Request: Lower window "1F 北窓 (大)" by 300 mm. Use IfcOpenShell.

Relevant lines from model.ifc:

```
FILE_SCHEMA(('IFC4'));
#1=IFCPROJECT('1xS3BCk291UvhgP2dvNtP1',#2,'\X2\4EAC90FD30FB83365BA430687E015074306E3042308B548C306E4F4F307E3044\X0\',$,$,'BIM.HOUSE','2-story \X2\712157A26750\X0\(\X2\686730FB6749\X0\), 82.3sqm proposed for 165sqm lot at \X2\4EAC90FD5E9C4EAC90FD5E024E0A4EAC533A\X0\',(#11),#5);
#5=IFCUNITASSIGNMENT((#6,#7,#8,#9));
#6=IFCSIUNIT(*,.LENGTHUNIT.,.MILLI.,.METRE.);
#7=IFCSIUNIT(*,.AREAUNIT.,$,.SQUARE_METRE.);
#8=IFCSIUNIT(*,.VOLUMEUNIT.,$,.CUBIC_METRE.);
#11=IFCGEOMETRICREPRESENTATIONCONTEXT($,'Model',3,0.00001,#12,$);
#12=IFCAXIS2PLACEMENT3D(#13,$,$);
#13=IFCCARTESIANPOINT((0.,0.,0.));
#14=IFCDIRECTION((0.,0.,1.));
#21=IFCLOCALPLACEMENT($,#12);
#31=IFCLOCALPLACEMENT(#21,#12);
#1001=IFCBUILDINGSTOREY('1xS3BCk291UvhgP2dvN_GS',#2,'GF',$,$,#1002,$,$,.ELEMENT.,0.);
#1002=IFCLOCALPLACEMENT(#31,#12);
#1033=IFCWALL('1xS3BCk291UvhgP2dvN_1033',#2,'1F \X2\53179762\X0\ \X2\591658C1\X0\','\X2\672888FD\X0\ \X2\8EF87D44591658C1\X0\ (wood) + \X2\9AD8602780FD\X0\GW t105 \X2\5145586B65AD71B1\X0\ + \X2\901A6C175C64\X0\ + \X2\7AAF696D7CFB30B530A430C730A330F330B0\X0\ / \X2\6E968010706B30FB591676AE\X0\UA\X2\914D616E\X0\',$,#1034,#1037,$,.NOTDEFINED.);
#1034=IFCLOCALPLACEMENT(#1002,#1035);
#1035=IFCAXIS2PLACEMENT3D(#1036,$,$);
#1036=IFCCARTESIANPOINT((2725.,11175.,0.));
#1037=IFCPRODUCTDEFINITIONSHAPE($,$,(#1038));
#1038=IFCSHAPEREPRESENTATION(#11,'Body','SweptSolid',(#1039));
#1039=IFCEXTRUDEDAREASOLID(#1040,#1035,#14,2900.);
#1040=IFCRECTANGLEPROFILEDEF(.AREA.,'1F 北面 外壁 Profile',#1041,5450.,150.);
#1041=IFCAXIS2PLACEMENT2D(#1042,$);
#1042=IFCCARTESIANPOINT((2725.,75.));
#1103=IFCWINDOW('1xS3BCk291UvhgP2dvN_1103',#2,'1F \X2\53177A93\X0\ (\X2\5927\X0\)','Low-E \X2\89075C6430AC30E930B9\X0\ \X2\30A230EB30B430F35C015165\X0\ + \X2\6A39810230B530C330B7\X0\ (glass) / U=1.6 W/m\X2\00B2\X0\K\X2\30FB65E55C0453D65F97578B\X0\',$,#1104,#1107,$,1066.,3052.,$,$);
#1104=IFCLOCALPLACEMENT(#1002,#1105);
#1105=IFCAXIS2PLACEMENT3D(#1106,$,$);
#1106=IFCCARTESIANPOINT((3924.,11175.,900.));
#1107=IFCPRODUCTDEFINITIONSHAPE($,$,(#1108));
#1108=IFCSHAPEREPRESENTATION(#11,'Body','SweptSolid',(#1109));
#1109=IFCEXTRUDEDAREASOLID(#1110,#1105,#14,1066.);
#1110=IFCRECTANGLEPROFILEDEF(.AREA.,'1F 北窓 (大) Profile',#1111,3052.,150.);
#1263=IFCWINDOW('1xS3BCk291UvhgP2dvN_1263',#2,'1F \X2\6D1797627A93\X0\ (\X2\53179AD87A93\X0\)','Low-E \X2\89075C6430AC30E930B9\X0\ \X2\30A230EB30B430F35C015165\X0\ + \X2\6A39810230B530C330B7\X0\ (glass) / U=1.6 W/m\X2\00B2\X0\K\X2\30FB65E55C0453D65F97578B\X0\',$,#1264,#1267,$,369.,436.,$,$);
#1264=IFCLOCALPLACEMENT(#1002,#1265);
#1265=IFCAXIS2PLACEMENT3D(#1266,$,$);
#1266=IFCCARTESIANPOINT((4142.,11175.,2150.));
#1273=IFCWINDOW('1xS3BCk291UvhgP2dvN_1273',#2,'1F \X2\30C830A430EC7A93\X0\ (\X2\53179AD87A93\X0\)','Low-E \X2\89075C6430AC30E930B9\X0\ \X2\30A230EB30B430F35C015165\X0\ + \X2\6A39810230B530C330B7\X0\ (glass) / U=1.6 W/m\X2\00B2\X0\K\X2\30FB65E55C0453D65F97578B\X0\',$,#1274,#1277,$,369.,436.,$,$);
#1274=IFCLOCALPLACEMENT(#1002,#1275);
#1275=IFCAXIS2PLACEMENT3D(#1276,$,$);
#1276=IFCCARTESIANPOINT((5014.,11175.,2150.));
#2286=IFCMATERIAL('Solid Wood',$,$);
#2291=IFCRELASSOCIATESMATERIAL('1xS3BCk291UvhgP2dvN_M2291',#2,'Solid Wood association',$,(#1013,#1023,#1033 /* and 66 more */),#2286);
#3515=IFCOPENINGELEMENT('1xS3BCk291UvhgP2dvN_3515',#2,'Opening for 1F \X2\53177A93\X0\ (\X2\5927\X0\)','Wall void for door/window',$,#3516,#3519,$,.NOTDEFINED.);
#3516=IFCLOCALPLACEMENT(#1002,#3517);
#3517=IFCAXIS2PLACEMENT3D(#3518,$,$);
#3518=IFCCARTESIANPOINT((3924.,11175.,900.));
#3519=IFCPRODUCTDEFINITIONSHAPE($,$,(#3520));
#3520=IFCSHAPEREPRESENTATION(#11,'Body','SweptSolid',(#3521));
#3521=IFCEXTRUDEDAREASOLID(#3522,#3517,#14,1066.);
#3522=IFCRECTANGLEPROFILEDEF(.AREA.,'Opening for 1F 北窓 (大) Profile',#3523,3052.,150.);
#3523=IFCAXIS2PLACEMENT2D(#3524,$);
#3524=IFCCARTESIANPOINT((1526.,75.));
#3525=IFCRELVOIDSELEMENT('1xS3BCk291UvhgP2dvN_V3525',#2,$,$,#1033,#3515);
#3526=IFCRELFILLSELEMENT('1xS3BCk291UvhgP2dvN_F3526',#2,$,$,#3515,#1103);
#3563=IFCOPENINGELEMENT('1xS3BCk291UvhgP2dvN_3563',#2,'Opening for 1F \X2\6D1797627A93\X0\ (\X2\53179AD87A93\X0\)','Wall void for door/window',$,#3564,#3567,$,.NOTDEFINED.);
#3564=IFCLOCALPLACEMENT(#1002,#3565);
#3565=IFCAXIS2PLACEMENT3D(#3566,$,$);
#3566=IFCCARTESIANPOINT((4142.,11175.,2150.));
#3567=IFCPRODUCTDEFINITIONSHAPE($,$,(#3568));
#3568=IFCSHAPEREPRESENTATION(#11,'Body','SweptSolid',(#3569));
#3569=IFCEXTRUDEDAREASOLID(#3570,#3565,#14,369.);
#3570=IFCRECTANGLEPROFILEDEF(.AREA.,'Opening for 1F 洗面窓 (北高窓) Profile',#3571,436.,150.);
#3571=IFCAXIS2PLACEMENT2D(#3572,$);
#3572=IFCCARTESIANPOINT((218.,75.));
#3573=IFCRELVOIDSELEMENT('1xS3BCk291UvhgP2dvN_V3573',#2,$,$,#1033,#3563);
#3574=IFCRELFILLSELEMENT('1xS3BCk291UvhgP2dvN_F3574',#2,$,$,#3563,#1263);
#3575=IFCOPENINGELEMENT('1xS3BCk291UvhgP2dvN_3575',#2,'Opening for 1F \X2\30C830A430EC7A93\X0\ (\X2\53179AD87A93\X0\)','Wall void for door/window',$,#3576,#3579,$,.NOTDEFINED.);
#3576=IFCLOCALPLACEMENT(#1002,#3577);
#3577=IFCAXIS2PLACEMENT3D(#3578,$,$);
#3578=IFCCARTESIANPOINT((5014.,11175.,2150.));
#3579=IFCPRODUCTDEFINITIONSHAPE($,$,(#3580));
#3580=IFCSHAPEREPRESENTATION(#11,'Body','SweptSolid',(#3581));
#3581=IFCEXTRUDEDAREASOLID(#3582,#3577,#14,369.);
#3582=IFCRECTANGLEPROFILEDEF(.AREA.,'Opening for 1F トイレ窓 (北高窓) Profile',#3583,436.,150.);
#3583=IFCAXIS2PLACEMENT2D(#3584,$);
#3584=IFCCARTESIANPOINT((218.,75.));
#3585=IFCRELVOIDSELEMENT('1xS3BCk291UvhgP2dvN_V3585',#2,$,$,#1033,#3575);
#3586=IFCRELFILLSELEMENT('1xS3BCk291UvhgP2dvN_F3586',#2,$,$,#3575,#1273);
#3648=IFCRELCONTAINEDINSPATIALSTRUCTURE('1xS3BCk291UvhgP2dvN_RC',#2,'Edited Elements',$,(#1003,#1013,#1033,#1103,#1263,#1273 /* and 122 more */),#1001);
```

```python
import numpy as np
import ifcopenshell
import ifcopenshell.api.geometry
import ifcopenshell.util.placement
import ifcopenshell.util.unit

model = ifcopenshell.open("model.ifc")
unit_scale = ifcopenshell.util.unit.calculate_unit_scale(model)

window = model.by_id(1103)
opening = window.FillsVoids[0].RelatingOpeningElement
dz = -0.3 / unit_scale

shift = np.array([0.0, 0.0, dz])
# The window is not placed relative to its opening, so move both.
for product in (opening, window):
    matrix = ifcopenshell.util.placement.get_local_placement(product.ObjectPlacement)
    matrix[:3, 3] += shift
    ifcopenshell.api.geometry.edit_object_placement(model, product=product, matrix=matrix, is_si=False)

print(f"moved by {dz * unit_scale:+.3f} m")

model.write("model_v2.ifc")
```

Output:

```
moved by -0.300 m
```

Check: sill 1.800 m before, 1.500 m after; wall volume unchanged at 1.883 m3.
